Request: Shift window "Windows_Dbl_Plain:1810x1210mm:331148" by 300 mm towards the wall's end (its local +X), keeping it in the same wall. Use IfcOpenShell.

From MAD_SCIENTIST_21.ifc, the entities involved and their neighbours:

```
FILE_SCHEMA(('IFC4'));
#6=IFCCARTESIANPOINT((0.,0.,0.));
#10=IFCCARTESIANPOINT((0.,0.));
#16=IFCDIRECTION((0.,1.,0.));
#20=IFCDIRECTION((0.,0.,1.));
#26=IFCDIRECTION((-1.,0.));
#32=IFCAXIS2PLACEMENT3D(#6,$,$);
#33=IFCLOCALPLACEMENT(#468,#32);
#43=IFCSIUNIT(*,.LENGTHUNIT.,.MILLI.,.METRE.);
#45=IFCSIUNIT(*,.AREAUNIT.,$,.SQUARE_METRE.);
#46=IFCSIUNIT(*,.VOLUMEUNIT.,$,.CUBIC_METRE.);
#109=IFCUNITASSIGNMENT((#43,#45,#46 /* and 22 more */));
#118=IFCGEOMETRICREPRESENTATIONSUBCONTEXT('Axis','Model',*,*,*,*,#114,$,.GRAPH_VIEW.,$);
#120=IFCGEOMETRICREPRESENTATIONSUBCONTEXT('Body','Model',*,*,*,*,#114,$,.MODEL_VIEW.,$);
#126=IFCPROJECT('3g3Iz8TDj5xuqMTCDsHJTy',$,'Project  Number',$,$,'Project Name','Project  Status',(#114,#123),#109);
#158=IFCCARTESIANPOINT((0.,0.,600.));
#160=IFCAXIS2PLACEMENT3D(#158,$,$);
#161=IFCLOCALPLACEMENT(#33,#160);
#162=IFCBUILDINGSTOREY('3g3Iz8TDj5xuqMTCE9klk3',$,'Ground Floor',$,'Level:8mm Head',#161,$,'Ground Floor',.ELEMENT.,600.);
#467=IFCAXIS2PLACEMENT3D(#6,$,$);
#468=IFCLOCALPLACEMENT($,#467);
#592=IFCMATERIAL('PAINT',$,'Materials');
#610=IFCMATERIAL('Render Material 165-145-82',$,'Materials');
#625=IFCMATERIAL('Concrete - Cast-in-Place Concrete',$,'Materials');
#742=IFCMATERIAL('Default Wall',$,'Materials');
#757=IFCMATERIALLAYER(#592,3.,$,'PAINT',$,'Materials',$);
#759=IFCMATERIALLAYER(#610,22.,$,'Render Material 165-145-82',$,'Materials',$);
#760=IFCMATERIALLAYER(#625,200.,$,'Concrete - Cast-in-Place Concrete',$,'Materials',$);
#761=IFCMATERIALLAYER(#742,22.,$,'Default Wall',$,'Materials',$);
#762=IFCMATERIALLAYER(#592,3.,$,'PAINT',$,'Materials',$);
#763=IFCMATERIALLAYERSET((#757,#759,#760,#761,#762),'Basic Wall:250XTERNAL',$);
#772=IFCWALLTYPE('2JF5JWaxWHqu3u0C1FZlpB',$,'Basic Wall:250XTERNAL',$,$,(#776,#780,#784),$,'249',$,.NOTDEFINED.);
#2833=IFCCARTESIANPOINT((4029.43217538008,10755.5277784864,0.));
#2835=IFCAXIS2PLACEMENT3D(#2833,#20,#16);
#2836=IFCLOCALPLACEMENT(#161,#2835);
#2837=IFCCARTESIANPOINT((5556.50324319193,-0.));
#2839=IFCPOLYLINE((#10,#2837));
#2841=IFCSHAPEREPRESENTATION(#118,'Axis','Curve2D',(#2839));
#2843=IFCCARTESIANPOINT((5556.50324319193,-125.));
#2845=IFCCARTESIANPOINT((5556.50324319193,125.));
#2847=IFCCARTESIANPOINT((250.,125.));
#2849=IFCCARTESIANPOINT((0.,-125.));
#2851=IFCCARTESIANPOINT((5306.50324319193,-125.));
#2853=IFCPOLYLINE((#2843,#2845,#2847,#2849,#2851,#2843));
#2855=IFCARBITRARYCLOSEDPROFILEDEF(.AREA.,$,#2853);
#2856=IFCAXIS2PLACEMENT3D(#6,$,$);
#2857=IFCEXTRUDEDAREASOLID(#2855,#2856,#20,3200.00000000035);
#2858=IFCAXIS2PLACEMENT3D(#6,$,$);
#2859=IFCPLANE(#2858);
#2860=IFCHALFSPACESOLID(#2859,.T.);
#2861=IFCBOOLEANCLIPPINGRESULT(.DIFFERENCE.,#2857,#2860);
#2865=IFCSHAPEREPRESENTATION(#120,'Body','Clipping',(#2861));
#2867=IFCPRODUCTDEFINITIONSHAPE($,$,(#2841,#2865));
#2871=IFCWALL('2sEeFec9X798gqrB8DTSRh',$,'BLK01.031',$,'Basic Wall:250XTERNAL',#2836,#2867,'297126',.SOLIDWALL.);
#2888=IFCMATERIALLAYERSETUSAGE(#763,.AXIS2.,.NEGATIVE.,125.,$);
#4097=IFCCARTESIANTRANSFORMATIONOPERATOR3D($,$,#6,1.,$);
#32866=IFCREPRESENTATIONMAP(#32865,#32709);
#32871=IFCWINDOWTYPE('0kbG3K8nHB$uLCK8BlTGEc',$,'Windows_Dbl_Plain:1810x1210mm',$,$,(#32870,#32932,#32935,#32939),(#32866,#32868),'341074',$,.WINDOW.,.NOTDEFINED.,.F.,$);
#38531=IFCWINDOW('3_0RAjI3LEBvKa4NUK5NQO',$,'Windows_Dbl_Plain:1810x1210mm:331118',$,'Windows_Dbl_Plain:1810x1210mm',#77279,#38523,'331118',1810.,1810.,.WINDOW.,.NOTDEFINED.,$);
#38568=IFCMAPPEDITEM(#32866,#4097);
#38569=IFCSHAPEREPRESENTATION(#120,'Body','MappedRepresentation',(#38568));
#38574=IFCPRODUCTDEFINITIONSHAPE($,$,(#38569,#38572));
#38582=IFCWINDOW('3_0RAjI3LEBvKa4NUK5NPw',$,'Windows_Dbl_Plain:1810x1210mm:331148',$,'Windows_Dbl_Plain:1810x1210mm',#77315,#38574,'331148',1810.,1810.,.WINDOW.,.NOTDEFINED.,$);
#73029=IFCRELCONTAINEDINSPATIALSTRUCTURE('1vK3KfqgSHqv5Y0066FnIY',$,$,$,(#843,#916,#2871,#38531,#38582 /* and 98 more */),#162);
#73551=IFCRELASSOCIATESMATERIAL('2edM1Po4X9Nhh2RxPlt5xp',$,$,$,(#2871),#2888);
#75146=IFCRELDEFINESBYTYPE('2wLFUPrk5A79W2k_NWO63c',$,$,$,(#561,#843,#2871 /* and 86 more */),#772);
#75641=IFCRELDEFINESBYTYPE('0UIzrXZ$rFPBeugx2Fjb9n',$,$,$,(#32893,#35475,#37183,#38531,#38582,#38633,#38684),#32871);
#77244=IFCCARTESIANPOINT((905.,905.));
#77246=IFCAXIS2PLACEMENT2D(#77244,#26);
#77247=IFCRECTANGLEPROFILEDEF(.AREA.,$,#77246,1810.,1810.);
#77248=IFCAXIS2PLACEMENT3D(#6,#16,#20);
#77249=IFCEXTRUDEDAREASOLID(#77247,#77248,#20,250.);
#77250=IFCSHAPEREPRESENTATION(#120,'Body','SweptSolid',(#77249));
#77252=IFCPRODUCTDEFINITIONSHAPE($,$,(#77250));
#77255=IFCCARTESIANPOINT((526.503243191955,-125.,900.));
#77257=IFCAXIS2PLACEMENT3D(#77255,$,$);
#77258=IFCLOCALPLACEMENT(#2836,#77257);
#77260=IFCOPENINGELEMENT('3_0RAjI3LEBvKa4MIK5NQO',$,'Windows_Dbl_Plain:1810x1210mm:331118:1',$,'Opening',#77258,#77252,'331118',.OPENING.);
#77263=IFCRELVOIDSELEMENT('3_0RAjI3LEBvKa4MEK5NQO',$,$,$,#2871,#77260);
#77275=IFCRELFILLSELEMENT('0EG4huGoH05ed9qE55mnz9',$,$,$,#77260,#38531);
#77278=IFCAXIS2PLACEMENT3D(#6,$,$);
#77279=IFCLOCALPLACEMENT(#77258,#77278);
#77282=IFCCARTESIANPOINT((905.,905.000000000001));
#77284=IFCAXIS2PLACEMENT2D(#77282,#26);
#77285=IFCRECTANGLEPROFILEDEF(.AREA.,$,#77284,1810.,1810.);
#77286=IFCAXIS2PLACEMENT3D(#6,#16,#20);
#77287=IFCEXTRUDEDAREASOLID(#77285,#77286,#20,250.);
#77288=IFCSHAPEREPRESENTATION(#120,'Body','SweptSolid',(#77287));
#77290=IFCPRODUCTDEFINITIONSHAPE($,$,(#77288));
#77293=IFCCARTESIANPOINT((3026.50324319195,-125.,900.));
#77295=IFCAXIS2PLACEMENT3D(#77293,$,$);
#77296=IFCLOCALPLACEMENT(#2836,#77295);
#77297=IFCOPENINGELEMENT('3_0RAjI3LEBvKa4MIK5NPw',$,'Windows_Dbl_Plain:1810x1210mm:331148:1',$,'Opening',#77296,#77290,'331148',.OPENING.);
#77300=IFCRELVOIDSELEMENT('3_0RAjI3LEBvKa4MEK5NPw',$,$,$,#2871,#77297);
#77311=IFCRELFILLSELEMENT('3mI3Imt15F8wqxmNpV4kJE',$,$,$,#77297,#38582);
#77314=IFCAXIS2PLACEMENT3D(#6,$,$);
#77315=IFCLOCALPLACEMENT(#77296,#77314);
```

```python
import ifcopenshell
import ifcopenshell.api.geometry
import ifcopenshell.util.placement
import ifcopenshell.util.unit

model = ifcopenshell.open("MAD_SCIENTIST_21.ifc")
unit_scale = ifcopenshell.util.unit.calculate_unit_scale(model)

window = model.by_guid("3_0RAjI3LEBvKa4NUK5NPw")
opening = window.FillsVoids[0].RelatingOpeningElement
wall = opening.VoidsElements[0].RelatingBuildingElement

wall_matrix = ifcopenshell.util.placement.get_local_placement(wall.ObjectPlacement)
shift = wall_matrix[:3, 0] * 0.3 / unit_scale
before = ifcopenshell.util.placement.get_local_placement(window.ObjectPlacement)[:3, 3].copy()

# The window is placed relative to its opening, so it follows when the opening moves.
matrix = ifcopenshell.util.placement.get_local_placement(opening.ObjectPlacement)
matrix[:3, 3] += shift
ifcopenshell.api.geometry.edit_object_placement(
    model, product=opening, matrix=matrix, is_si=False, should_transform_children=True
)

after = ifcopenshell.util.placement.get_local_placement(window.ObjectPlacement)[:3, 3]
print("window moved by", (after - before).round(3) + 0.0)

model.write("MAD_SCIENTIST_21_updated.ifc")
```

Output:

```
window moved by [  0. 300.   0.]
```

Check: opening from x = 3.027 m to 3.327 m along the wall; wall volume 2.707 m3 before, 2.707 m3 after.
